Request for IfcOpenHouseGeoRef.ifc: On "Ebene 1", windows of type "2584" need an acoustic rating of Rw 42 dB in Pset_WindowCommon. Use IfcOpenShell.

First a look at what the model holds.

```python
import ifcopenshell
import ifcopenshell.util.element

model = ifcopenshell.open("IfcOpenHouseGeoRef.ifc")
print(model.schema)
storey = next(s for s in model.by_type("IfcBuildingStorey") if s.Name == "Ebene 1")
windows = [e for e in ifcopenshell.util.element.get_decomposition(storey) if e.is_a("IfcWindow")]
seen = {}
for e in windows:
    element_type = ifcopenshell.util.element.get_type(e)
    key = (element_type.Name if element_type != e and element_type else None, ifcopenshell.util.element.get_pset(e, "Pset_WindowCommon", "AcousticRating"))
    seen[key] = seen.get(key, 0) + 1
for (name, value), count in sorted(seen.items(), key=str):
    print(count, "x", name, "|", value)
```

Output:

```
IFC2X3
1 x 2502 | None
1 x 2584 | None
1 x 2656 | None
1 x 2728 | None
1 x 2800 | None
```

```python
import ifcopenshell
import ifcopenshell.api.pset
import ifcopenshell.util.element

model = ifcopenshell.open("IfcOpenHouseGeoRef.ifc")

storey = next(s for s in model.by_type("IfcBuildingStorey") if s.Name == "Ebene 1")
windows = [e for e in ifcopenshell.util.element.get_decomposition(storey) if e.is_a("IfcWindow")]

count = 0
for e in windows:
    element_type = ifcopenshell.util.element.get_type(e)
    if element_type in (None, e) or element_type.Name != "2584":
        continue
    # add_pset returns the element's existing set when there is one.
    pset = ifcopenshell.api.pset.add_pset(model, product=e, name="Pset_WindowCommon")
    ifcopenshell.api.pset.edit_pset(model, pset=pset, properties={"AcousticRating": "Rw 42 dB"})
    count += 1

print(count, "windows updated")

model.write("IfcOpenHouseGeoRef_edited.ifc")
```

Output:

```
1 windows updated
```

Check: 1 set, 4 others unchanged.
